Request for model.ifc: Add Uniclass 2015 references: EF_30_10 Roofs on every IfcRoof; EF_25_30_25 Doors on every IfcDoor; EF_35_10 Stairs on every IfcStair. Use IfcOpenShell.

First a look at what the model holds.

```python
import ifcopenshell

model = ifcopenshell.open("model.ifc")
print(model.schema)
print("classifications:", [c.Name for c in model.by_type("IfcClassification")])
for ifc_class in ("IfcDoor", "IfcRoof", "IfcStair", "IfcWall", "IfcWindow"):
    print(ifc_class, len(model.by_type(ifc_class)))
```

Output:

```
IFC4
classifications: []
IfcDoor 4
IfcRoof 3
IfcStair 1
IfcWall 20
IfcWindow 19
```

```python
import ifcopenshell
import ifcopenshell.api.classification

model = ifcopenshell.open("model.ifc")

system = ifcopenshell.api.classification.add_classification(model, classification="Uniclass 2015")

codes = {
    "IfcRoof": ("EF_30_10", "Roofs"),
    "IfcDoor": ("EF_25_30_25", "Doors"),
    "IfcStair": ("EF_35_10", "Stairs"),
}
for ifc_class, (code, name) in codes.items():
    products = model.by_type(ifc_class)
    ifcopenshell.api.classification.add_reference(
        model, products=products, classification=system, identification=code, name=name
    )
    print(code, len(products))

model.write("model_edited.ifc")
```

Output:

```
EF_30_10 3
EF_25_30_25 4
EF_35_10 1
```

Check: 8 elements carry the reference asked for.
